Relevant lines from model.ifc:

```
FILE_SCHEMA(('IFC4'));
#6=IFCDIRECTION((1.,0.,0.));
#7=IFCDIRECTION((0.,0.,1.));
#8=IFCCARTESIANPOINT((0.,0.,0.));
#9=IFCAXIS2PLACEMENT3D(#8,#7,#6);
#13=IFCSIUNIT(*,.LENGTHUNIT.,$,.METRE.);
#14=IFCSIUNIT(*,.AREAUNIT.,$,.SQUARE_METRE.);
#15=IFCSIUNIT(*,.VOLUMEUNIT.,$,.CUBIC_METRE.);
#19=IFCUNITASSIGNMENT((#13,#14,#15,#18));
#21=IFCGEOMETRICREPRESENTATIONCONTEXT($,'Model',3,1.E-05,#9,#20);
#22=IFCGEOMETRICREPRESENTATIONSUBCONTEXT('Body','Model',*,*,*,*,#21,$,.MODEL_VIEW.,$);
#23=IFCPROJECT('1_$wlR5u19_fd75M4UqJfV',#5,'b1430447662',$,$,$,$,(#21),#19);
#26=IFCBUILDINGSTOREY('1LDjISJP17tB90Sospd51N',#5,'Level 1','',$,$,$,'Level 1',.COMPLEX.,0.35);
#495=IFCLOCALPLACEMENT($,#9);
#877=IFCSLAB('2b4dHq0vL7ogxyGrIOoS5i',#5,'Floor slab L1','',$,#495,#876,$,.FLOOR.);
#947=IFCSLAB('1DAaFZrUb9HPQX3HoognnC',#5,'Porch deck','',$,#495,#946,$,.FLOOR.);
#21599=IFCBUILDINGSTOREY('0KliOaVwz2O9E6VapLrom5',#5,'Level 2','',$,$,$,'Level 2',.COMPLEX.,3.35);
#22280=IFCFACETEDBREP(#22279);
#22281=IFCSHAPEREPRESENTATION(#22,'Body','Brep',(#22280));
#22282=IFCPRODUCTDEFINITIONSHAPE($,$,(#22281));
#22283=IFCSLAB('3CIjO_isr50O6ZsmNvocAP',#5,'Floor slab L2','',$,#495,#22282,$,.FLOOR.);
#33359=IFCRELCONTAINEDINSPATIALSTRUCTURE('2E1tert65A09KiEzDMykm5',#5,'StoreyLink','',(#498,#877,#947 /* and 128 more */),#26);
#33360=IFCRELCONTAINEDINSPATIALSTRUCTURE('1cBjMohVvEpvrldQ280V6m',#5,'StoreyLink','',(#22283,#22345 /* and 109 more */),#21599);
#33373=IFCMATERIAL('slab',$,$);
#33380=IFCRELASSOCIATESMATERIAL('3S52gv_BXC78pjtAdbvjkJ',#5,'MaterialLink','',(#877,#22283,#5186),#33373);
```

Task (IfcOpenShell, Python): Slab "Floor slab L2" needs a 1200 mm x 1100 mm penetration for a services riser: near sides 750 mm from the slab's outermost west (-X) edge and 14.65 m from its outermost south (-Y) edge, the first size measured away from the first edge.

```python
import numpy as np
import ifcopenshell
import ifcopenshell.api.feature
import ifcopenshell.api.geometry
import ifcopenshell.api.root
import ifcopenshell.geom
import ifcopenshell.util.placement
import ifcopenshell.util.representation
import ifcopenshell.util.shape
import ifcopenshell.util.unit

model = ifcopenshell.open("model.ifc")
unit_scale = ifcopenshell.util.unit.calculate_unit_scale(model)
settings = ifcopenshell.geom.settings()


def volume(element):
    """Net volume in cubic metres, openings subtracted."""
    shape = ifcopenshell.geom.create_shape(settings, element)
    return ifcopenshell.util.shape.get_volume(shape.geometry)


slab = model.by_id(22283)
before = volume(slab)

# Extent in the slab's own axes, in metres. The edges named are its -X and -Y sides.
slab_shape = ifcopenshell.geom.create_shape(settings, slab)
vertices = ifcopenshell.util.shape.get_vertices(slab_shape.geometry)
x_min, y_min, bottom = vertices.min(axis=0)
top = vertices[:, 2].max()

opening = ifcopenshell.api.root.create_entity(model, ifc_class="IfcOpeningElement", name="Services riser opening", predefined_type="OPENING")
context = ifcopenshell.util.representation.get_context(model, "Model", "Body", "MODEL_VIEW")
width, depth = 1.2, 1.1
outline = [(0.0, 0.0), (width, 0.0), (width, depth), (0.0, depth), (0.0, 0.0)]
# Overshoot both faces by 50 mm so the cut is clean.
shape = ifcopenshell.api.geometry.add_slab_representation(
    model, context=context, depth=top - bottom + 0.1, polyline=outline
)
ifcopenshell.api.geometry.assign_representation(model, product=opening, representation=shape)

matrix = ifcopenshell.util.placement.get_local_placement(slab.ObjectPlacement)
matrix[:, 3] = matrix @ np.append(np.array([x_min + 0.75, y_min + 14.65, bottom - 0.05]) / unit_scale, 1.0)
ifcopenshell.api.geometry.edit_object_placement(model, product=opening, matrix=matrix, is_si=False)
ifcopenshell.api.feature.add_feature(model, feature=opening, element=slab)

after = volume(slab)

print(f"slab volume {before:.3f} -> {after:.3f} m3")

model.write("model_rev.ifc")
```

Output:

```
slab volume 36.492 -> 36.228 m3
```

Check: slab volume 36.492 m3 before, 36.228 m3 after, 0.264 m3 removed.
